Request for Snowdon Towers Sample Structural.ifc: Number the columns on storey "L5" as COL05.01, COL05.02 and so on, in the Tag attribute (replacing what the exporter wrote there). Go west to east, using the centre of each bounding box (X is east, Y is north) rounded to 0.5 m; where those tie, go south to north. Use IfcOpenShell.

First a look at what the model holds.

```python
import ifcopenshell
import ifcopenshell.util.element
import ifcopenshell.util.placement

model = ifcopenshell.open("Snowdon Towers Sample Structural.ifc")
print(model.schema)
storey = next(s for s in model.by_type("IfcBuildingStorey") if s.Name == "L5")
columns = [e for e in ifcopenshell.util.element.get_decomposition(storey) if e.is_a("IfcColumn")]
for e in sorted(columns, key=lambda e: e.id()):
    origin = ifcopenshell.util.placement.get_local_placement(e.ObjectPlacement)[:3, 3]
    print(e.id(), e.Tag, e.Name, origin.round(2) + 0.0, sep=" | ")
```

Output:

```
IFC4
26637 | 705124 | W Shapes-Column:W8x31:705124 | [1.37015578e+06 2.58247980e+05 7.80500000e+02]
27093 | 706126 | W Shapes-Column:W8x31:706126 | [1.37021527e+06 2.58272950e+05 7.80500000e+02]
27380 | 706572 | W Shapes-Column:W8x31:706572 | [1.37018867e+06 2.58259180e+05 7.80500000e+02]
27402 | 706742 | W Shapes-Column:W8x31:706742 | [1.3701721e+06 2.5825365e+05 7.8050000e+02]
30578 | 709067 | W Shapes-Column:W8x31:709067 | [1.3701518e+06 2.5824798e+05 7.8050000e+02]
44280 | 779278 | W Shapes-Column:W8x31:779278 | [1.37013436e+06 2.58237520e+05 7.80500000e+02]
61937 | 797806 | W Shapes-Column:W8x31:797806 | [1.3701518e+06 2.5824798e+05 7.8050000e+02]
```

```python
import ifcopenshell
import ifcopenshell.geom
import ifcopenshell.util.element
import ifcopenshell.util.shape

model = ifcopenshell.open("Snowdon Towers Sample Structural.ifc")
settings = ifcopenshell.geom.settings()
settings.set("use-world-coords", True)


def centre(element):
    shape = ifcopenshell.geom.create_shape(settings, element)
    return ifcopenshell.util.shape.get_bbox_centroid(shape.geometry)


storey = next(s for s in model.by_type("IfcBuildingStorey") if s.Name == "L5")
columns = [e for e in ifcopenshell.util.element.get_decomposition(storey) if e.is_a("IfcColumn")]

# Insertion points can sit at a corner or the storey origin, so sort by the geometry (in metres).
centres = {e: centre(e) for e in columns}
columns.sort(key=lambda e: (round(centres[e][0] / 0.5), centres[e][1]))

for i, e in enumerate(columns, start=1):
    number = f"COL05.{i:02d}"
    e.Tag = number
    print(e.id(), number)

model.write("Snowdon Towers Sample Structural_edited.ifc")
```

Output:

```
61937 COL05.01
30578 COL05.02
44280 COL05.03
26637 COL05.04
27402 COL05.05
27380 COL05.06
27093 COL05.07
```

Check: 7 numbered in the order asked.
